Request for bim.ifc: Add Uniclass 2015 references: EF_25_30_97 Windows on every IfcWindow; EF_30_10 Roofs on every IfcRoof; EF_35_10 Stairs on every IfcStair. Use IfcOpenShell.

First a look at what the model holds.

```python
import ifcopenshell

model = ifcopenshell.open("bim.ifc")
print(model.schema)
print("classifications:", [c.Name for c in model.by_type("IfcClassification")])
for ifc_class in ("IfcDoor", "IfcRoof", "IfcStair", "IfcWall", "IfcWindow"):
    print(ifc_class, len(model.by_type(ifc_class)))
```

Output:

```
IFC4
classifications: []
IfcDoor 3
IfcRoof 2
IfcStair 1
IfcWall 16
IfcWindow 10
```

```python
import ifcopenshell
import ifcopenshell.api.classification

model = ifcopenshell.open("bim.ifc")

system = ifcopenshell.api.classification.add_classification(model, classification="Uniclass 2015")

codes = {
    "IfcWindow": ("EF_25_30_97", "Windows"),
    "IfcRoof": ("EF_30_10", "Roofs"),
    "IfcStair": ("EF_35_10", "Stairs"),
}
for ifc_class, (code, name) in codes.items():
    products = model.by_type(ifc_class)
    ifcopenshell.api.classification.add_reference(
        model, products=products, classification=system, identification=code, name=name
    )
    print(code, len(products))

model.write("bim-out.ifc")
```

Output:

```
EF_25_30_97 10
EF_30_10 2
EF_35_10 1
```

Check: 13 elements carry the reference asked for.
